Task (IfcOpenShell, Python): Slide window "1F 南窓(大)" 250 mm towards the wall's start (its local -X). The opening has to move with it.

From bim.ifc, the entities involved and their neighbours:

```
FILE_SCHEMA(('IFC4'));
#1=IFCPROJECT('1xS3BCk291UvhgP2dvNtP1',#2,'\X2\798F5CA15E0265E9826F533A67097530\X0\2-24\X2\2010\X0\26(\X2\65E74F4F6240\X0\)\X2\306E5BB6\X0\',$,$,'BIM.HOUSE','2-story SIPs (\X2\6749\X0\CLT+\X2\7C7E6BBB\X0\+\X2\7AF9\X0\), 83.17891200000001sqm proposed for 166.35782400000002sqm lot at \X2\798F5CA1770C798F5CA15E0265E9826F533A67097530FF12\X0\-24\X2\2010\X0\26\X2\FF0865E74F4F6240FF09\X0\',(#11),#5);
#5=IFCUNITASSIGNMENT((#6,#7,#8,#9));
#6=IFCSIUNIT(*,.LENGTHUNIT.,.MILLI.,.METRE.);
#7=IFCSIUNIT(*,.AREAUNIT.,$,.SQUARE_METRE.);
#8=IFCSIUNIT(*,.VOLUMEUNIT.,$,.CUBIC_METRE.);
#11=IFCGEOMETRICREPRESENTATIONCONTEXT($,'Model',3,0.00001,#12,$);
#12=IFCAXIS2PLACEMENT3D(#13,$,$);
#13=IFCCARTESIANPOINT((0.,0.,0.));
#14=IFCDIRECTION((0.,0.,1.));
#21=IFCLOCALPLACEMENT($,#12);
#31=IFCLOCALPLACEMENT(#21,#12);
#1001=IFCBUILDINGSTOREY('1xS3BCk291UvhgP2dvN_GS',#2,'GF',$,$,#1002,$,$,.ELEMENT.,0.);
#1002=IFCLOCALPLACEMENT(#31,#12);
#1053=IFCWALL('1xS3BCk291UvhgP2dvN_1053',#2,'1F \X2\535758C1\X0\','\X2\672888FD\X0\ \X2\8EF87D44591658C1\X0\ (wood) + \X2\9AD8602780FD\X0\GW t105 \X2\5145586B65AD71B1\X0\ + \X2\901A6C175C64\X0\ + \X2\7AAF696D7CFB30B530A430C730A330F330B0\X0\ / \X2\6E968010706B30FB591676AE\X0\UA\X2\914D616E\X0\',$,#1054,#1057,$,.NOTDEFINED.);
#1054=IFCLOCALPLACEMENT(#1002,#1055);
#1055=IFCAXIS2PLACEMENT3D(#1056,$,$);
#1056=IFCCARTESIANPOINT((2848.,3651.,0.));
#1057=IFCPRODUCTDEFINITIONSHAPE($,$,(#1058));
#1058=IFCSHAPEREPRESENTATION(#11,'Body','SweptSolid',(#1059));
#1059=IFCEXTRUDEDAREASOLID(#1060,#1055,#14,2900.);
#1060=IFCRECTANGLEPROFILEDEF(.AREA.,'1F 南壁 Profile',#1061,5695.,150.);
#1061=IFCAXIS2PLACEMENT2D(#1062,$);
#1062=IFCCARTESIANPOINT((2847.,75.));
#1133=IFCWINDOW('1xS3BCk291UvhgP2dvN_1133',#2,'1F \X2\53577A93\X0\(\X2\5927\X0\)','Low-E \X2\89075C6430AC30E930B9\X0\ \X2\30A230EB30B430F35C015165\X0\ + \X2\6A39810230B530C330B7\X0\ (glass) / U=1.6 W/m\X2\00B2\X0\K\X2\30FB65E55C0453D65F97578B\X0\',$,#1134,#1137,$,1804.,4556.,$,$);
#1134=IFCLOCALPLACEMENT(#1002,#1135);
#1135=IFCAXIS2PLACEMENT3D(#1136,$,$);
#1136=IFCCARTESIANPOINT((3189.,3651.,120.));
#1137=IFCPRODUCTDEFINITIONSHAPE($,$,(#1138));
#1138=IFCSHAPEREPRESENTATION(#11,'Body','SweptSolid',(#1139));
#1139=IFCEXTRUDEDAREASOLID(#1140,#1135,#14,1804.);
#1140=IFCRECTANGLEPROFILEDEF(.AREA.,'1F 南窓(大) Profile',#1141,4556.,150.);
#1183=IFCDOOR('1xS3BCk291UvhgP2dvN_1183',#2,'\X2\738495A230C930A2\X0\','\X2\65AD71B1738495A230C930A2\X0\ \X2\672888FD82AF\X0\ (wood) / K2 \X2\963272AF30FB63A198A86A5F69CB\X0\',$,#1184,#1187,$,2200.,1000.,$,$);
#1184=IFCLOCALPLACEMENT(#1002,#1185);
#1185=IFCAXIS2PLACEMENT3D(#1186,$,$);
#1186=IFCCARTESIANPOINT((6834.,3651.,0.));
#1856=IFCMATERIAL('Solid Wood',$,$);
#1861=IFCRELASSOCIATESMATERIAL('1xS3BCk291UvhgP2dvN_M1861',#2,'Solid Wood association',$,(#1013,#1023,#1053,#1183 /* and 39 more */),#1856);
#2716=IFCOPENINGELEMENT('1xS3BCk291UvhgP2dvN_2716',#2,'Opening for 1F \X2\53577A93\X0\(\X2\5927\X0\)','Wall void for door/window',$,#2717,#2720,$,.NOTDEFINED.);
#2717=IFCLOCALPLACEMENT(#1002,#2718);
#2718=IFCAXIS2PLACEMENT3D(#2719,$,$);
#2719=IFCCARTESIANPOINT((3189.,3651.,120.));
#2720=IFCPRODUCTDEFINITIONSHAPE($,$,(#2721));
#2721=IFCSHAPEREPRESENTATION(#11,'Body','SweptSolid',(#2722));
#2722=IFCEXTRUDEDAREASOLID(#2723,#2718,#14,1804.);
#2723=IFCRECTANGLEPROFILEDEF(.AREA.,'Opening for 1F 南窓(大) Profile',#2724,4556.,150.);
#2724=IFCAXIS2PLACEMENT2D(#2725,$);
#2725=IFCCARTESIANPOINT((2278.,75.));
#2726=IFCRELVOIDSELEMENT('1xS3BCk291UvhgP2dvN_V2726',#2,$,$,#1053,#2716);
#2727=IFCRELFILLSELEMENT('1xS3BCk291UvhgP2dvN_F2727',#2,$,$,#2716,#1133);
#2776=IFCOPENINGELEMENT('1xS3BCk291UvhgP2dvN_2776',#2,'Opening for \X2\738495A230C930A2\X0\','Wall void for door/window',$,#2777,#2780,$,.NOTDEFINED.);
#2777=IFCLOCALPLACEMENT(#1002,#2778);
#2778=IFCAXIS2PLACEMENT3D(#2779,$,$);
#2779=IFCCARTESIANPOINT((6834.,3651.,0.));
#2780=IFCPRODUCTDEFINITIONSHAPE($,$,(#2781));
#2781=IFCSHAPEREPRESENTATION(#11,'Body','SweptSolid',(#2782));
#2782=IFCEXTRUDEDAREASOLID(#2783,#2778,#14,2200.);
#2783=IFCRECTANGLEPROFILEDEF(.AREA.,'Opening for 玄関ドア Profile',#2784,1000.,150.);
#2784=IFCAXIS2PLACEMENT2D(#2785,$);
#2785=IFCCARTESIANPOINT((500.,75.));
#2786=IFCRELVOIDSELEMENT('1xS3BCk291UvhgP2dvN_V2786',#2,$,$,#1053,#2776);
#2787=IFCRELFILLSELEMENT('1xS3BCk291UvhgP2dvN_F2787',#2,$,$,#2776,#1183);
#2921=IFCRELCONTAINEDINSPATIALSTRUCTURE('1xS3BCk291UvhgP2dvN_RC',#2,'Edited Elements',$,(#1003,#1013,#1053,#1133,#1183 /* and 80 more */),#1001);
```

```python
import ifcopenshell
import ifcopenshell.api.geometry
import ifcopenshell.util.placement
import ifcopenshell.util.unit

model = ifcopenshell.open("bim.ifc")
unit_scale = ifcopenshell.util.unit.calculate_unit_scale(model)

window = model.by_guid("1xS3BCk291UvhgP2dvN_1133")
opening = window.FillsVoids[0].RelatingOpeningElement
wall = opening.VoidsElements[0].RelatingBuildingElement

wall_matrix = ifcopenshell.util.placement.get_local_placement(wall.ObjectPlacement)
shift = wall_matrix[:3, 0] * -0.25 / unit_scale
before = ifcopenshell.util.placement.get_local_placement(window.ObjectPlacement)[:3, 3].copy()

# The window is not placed relative to its opening, so move both.
for product in (opening, window):
    matrix = ifcopenshell.util.placement.get_local_placement(product.ObjectPlacement)
    matrix[:3, 3] += shift
    ifcopenshell.api.geometry.edit_object_placement(model, product=product, matrix=matrix, is_si=False)

after = ifcopenshell.util.placement.get_local_placement(window.ObjectPlacement)[:3, 3]
print("window moved by", (after - before).round(3) + 0.0)

model.write("bim_v2.ifc")
```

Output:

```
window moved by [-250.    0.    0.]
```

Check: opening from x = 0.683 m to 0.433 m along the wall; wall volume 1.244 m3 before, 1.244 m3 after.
